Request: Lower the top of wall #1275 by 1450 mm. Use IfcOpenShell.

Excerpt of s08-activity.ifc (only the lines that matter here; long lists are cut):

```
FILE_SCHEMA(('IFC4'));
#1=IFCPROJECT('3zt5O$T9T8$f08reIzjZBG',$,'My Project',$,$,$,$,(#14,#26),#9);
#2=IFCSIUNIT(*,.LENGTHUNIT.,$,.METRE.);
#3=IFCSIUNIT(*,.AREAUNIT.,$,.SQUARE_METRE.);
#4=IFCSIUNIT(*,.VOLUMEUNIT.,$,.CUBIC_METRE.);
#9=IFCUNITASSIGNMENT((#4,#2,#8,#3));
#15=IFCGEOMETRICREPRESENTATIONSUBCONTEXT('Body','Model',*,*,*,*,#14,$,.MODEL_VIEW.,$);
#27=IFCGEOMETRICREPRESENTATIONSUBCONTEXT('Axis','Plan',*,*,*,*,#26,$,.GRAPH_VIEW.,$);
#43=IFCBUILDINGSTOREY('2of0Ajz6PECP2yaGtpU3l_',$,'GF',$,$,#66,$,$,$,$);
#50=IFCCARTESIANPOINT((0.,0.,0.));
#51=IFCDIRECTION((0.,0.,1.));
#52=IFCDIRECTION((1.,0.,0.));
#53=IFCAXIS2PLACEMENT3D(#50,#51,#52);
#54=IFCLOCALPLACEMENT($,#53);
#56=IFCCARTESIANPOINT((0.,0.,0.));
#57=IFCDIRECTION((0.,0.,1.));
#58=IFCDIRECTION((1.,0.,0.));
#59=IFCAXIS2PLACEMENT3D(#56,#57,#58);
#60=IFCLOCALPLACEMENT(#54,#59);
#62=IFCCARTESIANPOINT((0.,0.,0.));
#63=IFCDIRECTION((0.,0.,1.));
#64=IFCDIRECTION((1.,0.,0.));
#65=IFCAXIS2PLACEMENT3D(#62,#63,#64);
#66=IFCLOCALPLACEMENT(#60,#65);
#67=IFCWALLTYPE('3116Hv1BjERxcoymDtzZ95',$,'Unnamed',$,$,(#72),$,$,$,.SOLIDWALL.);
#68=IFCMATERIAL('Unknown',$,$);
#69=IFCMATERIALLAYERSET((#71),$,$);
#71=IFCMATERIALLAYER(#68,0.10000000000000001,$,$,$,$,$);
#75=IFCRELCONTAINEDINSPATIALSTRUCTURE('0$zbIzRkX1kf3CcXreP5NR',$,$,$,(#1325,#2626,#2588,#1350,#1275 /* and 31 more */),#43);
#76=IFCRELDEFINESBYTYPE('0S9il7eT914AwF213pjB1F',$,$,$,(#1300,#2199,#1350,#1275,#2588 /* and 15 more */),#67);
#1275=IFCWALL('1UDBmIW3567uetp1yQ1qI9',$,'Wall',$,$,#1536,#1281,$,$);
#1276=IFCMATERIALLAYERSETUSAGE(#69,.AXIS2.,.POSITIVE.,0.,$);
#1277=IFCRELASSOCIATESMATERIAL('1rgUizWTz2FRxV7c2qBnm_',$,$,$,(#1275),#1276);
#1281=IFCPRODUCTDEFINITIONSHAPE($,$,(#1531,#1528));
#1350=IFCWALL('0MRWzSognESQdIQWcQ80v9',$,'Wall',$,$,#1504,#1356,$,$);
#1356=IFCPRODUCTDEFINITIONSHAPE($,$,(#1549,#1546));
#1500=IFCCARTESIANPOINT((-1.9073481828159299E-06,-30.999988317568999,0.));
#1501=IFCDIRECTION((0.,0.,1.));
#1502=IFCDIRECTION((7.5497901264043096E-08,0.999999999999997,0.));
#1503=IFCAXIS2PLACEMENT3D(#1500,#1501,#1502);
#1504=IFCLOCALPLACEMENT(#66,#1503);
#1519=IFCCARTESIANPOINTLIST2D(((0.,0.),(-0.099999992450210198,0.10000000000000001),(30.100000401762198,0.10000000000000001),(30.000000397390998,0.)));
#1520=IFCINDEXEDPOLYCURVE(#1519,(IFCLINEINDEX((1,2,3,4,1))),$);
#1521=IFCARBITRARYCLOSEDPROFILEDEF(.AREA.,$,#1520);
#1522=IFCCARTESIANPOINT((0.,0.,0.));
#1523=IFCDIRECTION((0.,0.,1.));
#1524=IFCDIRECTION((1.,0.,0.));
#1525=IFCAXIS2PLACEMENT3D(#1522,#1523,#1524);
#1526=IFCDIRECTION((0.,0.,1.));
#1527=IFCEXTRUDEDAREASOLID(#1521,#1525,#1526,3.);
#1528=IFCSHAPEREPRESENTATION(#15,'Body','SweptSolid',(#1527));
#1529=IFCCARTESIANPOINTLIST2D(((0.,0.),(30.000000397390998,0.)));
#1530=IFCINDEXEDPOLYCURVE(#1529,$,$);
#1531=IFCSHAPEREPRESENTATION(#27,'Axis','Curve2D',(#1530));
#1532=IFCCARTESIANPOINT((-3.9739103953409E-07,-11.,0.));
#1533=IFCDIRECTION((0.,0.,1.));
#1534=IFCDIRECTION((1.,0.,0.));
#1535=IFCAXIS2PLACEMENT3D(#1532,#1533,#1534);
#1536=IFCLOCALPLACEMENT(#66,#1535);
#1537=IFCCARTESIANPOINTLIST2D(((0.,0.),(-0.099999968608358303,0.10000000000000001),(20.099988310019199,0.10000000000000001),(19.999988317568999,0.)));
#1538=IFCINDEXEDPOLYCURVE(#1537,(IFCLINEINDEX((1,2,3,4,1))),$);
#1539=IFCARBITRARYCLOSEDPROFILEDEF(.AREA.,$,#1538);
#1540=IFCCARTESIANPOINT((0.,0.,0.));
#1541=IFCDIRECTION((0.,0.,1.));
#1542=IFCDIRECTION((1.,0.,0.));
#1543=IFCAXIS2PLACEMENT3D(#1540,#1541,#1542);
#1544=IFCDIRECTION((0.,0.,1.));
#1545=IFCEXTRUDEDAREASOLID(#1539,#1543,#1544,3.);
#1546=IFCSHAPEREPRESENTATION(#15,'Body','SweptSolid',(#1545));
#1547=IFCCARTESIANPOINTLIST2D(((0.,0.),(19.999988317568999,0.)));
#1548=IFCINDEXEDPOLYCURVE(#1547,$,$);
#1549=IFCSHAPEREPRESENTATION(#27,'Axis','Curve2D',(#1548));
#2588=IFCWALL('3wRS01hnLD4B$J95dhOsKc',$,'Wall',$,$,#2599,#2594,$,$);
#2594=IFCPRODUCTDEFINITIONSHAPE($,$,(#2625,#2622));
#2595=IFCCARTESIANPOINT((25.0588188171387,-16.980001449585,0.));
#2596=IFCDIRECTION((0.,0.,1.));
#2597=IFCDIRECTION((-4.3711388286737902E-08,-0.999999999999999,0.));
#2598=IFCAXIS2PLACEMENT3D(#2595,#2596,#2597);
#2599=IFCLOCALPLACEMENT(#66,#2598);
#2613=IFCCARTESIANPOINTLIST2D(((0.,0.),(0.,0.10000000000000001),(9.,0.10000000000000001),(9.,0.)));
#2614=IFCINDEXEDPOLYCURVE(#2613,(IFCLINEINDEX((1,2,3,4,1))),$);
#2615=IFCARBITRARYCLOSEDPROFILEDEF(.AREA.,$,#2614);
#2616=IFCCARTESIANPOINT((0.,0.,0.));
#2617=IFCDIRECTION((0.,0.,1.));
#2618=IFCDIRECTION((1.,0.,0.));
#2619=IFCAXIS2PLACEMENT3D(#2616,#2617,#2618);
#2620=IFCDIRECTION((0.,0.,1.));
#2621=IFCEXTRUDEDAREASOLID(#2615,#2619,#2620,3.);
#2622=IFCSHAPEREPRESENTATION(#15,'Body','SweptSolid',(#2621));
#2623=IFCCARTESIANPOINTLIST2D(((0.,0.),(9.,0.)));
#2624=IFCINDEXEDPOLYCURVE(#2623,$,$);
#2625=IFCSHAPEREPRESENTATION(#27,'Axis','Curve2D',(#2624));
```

```python
import ifcopenshell
import ifcopenshell.geom
import ifcopenshell.util.representation
import ifcopenshell.util.shape

model = ifcopenshell.open("s08-activity.ifc")
settings = ifcopenshell.geom.settings()


def volume(element):
    """Net volume in cubic metres, openings subtracted."""
    shape = ifcopenshell.geom.create_shape(settings, element)
    return ifcopenshell.util.shape.get_volume(shape.geometry)


wall = model.by_id(1275)
before = volume(wall)

body = ifcopenshell.util.representation.get_representation(wall, "Model", "Body")
solid = body.Items[0]
old_height = solid.Depth
solid.Depth -= 1.45
after = volume(wall)

print(f"height {old_height:g} -> {solid.Depth:g}, volume {before:.3f} -> {after:.3f} m3")

model.write("s08-activity_updated.ifc")
```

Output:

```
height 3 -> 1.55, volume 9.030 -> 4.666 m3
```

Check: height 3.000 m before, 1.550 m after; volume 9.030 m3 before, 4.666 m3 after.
